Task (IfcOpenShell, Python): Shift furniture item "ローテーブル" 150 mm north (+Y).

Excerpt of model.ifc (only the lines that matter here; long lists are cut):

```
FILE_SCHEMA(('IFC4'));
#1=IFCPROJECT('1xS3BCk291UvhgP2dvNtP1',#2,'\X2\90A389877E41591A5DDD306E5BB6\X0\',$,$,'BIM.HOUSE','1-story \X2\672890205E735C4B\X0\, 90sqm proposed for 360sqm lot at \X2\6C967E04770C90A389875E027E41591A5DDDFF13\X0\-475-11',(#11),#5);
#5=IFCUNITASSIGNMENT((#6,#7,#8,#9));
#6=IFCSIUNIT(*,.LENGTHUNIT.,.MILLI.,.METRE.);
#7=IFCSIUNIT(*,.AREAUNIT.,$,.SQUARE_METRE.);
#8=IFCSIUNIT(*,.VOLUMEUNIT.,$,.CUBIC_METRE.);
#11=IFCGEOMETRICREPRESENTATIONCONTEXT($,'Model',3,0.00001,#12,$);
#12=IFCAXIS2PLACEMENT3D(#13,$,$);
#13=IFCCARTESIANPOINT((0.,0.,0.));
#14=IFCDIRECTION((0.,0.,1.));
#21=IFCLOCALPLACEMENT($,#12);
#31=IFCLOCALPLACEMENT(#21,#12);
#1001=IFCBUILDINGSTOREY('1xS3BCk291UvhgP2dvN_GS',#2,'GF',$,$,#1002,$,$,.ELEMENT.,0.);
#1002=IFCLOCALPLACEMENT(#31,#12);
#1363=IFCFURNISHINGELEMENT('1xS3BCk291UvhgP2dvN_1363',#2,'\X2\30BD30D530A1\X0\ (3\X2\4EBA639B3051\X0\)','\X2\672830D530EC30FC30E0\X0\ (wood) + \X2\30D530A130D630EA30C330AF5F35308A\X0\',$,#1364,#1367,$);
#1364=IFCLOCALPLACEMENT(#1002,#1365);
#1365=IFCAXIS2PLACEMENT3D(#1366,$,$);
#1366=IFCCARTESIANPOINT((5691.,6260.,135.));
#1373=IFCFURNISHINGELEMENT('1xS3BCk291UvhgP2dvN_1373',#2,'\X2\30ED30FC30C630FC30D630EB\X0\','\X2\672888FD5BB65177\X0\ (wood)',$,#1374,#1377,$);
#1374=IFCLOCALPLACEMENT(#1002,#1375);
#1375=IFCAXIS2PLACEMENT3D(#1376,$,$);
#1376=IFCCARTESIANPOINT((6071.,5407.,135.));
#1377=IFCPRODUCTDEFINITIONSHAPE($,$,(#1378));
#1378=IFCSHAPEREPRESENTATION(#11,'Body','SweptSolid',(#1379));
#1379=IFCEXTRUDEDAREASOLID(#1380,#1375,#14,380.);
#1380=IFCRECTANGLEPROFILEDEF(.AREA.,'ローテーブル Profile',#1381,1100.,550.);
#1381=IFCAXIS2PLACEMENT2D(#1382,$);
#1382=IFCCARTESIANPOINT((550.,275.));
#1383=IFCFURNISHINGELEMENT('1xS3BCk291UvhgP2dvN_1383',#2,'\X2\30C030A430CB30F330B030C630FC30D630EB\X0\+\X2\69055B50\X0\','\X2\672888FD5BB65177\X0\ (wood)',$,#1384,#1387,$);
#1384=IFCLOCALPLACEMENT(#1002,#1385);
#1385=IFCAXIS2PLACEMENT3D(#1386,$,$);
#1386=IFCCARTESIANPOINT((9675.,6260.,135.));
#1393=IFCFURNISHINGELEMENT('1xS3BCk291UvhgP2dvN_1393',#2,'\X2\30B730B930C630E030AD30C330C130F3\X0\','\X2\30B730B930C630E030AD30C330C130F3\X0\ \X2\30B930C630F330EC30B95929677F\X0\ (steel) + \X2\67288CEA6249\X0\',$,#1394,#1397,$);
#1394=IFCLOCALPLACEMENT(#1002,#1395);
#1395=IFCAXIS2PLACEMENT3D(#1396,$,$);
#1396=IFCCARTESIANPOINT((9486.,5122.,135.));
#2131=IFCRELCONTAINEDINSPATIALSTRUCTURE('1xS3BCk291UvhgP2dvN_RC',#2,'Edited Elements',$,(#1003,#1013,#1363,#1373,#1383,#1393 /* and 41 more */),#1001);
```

```python
import ifcopenshell
import ifcopenshell.api.geometry
import ifcopenshell.util.placement
import ifcopenshell.util.unit

model = ifcopenshell.open("model.ifc")
unit_scale = ifcopenshell.util.unit.calculate_unit_scale(model)

item = model.by_id(1373)
matrix = ifcopenshell.util.placement.get_local_placement(item.ObjectPlacement)
matrix[1, 3] += 0.15 / unit_scale
ifcopenshell.api.geometry.edit_object_placement(model, product=item, matrix=matrix, is_si=False)

print(ifcopenshell.util.placement.get_local_placement(item.ObjectPlacement).round(3) + 0.0)

model.write("model_edited.ifc")
```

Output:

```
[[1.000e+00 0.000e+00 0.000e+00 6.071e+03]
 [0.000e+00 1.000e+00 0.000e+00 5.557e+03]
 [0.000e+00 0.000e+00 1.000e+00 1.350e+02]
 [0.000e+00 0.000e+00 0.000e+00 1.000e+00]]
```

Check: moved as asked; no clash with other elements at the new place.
